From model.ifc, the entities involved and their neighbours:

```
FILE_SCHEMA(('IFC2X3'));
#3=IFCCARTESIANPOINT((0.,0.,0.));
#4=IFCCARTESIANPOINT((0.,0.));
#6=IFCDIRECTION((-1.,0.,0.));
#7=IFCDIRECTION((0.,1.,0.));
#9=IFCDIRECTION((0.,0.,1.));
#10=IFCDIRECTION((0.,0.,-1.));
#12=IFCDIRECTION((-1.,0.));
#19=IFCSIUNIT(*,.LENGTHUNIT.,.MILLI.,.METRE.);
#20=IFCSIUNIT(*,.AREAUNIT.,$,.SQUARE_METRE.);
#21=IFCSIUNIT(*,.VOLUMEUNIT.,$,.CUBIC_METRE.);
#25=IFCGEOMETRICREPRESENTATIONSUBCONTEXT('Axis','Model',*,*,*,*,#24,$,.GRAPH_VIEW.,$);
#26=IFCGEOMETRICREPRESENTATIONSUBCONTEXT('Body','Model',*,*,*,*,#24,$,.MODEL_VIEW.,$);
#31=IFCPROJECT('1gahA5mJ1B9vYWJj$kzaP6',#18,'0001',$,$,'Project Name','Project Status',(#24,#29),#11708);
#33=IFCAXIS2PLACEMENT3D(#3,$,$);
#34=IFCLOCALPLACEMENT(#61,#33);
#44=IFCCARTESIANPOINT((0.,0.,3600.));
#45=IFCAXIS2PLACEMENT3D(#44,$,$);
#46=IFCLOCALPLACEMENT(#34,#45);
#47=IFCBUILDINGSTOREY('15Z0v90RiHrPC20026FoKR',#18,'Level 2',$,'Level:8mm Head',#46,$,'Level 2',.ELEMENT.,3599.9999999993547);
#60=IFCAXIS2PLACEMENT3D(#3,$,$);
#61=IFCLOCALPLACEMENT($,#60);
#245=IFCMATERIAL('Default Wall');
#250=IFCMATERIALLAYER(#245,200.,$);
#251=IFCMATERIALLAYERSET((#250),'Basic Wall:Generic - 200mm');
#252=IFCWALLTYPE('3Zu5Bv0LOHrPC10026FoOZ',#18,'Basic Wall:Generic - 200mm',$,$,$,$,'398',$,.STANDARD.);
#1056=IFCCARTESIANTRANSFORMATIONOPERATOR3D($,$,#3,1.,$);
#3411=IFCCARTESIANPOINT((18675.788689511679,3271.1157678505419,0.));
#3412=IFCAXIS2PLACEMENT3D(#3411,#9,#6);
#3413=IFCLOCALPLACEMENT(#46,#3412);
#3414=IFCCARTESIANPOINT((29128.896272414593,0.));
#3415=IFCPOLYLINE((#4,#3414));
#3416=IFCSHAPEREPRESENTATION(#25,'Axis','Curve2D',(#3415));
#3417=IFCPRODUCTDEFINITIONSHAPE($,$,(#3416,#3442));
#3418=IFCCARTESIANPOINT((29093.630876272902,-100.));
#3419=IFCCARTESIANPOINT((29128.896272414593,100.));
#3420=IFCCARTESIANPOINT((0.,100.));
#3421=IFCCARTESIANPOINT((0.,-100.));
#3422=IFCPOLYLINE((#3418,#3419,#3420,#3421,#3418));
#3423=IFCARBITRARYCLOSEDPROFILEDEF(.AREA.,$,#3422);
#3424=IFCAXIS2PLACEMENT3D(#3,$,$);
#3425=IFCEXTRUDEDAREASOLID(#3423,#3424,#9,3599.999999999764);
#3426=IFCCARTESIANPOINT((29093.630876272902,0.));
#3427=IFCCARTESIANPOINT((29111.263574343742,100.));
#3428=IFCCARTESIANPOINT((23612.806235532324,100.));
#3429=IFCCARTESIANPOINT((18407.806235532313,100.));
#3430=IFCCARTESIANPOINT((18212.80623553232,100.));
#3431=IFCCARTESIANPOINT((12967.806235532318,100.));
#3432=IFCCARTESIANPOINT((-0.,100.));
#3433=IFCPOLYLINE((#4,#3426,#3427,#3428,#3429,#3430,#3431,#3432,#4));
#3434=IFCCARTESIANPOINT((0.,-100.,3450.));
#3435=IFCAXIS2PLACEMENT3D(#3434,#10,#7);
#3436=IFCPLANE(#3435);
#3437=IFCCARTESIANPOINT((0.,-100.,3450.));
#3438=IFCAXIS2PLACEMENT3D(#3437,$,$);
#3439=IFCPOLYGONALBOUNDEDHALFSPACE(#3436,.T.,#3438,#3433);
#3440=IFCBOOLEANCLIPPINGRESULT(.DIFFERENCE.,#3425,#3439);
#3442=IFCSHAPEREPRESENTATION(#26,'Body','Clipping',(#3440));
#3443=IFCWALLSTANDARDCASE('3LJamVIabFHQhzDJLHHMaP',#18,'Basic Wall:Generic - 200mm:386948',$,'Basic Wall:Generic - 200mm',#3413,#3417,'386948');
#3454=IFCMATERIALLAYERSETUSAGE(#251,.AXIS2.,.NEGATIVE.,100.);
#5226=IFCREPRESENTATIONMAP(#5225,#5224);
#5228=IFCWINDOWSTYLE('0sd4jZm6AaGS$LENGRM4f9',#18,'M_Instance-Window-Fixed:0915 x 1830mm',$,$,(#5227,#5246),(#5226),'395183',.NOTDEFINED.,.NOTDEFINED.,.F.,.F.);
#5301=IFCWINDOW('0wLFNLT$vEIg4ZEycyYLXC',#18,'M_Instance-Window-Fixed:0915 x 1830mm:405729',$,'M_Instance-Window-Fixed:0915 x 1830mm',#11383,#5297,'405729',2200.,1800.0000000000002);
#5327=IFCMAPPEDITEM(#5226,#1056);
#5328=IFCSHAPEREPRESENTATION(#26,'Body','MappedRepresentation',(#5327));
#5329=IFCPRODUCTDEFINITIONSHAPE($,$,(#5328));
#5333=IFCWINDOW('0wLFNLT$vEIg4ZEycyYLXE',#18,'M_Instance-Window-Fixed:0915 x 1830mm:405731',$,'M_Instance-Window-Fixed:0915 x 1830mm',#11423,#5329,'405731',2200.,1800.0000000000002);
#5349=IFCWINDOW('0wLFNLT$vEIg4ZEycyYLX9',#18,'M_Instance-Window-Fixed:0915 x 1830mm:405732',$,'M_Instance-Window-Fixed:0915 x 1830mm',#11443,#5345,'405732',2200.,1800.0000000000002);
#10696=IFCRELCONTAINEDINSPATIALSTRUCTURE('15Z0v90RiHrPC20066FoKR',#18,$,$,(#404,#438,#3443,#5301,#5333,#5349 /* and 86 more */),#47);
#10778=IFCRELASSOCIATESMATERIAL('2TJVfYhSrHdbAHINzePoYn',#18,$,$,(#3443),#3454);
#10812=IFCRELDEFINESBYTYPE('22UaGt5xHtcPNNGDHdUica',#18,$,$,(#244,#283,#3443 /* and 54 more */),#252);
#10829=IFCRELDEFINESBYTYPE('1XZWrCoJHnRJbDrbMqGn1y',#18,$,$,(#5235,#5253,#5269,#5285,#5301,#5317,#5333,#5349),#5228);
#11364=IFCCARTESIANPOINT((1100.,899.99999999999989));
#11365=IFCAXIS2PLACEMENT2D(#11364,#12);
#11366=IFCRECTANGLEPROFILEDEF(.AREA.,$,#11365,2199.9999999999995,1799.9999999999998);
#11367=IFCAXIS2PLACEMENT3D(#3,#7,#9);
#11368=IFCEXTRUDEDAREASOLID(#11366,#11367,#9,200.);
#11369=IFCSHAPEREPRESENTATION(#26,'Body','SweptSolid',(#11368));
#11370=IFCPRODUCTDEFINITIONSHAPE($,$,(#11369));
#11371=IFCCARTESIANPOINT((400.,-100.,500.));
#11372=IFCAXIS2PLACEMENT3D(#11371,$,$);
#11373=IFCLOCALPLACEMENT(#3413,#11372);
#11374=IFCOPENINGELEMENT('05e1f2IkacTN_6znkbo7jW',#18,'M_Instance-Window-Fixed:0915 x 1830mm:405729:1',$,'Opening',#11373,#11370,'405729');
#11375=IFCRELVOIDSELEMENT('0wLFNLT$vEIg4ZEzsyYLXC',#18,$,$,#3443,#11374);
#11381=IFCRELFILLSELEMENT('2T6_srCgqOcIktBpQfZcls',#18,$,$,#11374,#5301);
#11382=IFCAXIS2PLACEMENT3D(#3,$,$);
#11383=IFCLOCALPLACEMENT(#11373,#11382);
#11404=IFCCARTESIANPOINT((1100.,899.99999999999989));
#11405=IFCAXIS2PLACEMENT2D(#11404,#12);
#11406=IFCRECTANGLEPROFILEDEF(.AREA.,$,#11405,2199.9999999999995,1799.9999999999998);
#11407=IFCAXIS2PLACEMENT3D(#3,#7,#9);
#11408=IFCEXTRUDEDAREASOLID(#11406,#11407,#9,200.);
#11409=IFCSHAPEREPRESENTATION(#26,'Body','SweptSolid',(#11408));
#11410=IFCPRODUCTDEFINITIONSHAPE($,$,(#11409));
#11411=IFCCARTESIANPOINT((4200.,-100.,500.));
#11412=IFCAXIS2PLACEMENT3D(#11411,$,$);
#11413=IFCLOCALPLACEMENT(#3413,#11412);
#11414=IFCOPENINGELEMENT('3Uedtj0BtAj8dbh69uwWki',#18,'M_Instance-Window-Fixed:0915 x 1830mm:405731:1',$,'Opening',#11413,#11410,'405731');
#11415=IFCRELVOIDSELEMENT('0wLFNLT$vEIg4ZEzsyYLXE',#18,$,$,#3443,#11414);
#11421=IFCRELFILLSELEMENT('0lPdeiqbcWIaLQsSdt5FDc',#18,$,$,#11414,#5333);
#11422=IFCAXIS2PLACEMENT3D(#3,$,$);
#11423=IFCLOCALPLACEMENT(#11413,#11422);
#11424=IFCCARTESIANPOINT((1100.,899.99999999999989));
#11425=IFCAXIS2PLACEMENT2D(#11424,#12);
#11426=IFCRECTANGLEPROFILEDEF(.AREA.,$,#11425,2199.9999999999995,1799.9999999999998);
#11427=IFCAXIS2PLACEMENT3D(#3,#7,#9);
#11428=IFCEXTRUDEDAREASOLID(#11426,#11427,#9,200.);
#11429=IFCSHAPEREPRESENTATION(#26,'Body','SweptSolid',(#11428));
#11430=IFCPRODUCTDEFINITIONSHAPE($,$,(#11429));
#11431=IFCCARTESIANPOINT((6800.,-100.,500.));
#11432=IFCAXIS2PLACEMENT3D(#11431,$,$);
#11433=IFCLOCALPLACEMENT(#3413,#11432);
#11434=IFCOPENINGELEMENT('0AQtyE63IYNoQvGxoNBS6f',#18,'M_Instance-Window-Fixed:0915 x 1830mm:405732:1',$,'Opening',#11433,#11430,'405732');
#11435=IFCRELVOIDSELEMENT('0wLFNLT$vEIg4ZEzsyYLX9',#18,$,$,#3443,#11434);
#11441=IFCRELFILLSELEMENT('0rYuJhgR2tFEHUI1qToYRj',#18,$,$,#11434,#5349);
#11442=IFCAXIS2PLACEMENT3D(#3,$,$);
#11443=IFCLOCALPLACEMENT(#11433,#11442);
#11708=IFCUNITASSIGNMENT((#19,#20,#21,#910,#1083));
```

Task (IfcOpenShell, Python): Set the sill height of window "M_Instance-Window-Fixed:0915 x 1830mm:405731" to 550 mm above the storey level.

```python
import numpy as np
import ifcopenshell
import ifcopenshell.api.geometry
import ifcopenshell.geom
import ifcopenshell.util.element
import ifcopenshell.util.placement
import ifcopenshell.util.shape
import ifcopenshell.util.unit

model = ifcopenshell.open("model.ifc")
unit_scale = ifcopenshell.util.unit.calculate_unit_scale(model)

window = model.by_guid("0wLFNLT$vEIg4ZEycyYLXE")
opening = window.FillsVoids[0].RelatingOpeningElement
storey = ifcopenshell.util.element.get_container(window, ifc_class="IfcBuildingStorey")
level = ifcopenshell.util.placement.get_local_placement(storey.ObjectPlacement)[2, 3]

# The opening's origin need not be at the sill, so measure its lowest point.
shape = ifcopenshell.geom.create_shape(ifcopenshell.geom.settings(), opening)
bottom = ifcopenshell.util.shape.get_shape_bottom_elevation(shape, shape.geometry) / unit_scale
dz = level + 0.55 / unit_scale - bottom

shift = np.array([0.0, 0.0, dz])
# The window is placed relative to its opening, so it follows when the opening moves.
matrix = ifcopenshell.util.placement.get_local_placement(opening.ObjectPlacement)
matrix[:3, 3] += shift
ifcopenshell.api.geometry.edit_object_placement(
    model, product=opening, matrix=matrix, is_si=False, should_transform_children=True
)

print(f"moved by {dz * unit_scale:+.3f} m")

model.write("model_edited.ifc")
```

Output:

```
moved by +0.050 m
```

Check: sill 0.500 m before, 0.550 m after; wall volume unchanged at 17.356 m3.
